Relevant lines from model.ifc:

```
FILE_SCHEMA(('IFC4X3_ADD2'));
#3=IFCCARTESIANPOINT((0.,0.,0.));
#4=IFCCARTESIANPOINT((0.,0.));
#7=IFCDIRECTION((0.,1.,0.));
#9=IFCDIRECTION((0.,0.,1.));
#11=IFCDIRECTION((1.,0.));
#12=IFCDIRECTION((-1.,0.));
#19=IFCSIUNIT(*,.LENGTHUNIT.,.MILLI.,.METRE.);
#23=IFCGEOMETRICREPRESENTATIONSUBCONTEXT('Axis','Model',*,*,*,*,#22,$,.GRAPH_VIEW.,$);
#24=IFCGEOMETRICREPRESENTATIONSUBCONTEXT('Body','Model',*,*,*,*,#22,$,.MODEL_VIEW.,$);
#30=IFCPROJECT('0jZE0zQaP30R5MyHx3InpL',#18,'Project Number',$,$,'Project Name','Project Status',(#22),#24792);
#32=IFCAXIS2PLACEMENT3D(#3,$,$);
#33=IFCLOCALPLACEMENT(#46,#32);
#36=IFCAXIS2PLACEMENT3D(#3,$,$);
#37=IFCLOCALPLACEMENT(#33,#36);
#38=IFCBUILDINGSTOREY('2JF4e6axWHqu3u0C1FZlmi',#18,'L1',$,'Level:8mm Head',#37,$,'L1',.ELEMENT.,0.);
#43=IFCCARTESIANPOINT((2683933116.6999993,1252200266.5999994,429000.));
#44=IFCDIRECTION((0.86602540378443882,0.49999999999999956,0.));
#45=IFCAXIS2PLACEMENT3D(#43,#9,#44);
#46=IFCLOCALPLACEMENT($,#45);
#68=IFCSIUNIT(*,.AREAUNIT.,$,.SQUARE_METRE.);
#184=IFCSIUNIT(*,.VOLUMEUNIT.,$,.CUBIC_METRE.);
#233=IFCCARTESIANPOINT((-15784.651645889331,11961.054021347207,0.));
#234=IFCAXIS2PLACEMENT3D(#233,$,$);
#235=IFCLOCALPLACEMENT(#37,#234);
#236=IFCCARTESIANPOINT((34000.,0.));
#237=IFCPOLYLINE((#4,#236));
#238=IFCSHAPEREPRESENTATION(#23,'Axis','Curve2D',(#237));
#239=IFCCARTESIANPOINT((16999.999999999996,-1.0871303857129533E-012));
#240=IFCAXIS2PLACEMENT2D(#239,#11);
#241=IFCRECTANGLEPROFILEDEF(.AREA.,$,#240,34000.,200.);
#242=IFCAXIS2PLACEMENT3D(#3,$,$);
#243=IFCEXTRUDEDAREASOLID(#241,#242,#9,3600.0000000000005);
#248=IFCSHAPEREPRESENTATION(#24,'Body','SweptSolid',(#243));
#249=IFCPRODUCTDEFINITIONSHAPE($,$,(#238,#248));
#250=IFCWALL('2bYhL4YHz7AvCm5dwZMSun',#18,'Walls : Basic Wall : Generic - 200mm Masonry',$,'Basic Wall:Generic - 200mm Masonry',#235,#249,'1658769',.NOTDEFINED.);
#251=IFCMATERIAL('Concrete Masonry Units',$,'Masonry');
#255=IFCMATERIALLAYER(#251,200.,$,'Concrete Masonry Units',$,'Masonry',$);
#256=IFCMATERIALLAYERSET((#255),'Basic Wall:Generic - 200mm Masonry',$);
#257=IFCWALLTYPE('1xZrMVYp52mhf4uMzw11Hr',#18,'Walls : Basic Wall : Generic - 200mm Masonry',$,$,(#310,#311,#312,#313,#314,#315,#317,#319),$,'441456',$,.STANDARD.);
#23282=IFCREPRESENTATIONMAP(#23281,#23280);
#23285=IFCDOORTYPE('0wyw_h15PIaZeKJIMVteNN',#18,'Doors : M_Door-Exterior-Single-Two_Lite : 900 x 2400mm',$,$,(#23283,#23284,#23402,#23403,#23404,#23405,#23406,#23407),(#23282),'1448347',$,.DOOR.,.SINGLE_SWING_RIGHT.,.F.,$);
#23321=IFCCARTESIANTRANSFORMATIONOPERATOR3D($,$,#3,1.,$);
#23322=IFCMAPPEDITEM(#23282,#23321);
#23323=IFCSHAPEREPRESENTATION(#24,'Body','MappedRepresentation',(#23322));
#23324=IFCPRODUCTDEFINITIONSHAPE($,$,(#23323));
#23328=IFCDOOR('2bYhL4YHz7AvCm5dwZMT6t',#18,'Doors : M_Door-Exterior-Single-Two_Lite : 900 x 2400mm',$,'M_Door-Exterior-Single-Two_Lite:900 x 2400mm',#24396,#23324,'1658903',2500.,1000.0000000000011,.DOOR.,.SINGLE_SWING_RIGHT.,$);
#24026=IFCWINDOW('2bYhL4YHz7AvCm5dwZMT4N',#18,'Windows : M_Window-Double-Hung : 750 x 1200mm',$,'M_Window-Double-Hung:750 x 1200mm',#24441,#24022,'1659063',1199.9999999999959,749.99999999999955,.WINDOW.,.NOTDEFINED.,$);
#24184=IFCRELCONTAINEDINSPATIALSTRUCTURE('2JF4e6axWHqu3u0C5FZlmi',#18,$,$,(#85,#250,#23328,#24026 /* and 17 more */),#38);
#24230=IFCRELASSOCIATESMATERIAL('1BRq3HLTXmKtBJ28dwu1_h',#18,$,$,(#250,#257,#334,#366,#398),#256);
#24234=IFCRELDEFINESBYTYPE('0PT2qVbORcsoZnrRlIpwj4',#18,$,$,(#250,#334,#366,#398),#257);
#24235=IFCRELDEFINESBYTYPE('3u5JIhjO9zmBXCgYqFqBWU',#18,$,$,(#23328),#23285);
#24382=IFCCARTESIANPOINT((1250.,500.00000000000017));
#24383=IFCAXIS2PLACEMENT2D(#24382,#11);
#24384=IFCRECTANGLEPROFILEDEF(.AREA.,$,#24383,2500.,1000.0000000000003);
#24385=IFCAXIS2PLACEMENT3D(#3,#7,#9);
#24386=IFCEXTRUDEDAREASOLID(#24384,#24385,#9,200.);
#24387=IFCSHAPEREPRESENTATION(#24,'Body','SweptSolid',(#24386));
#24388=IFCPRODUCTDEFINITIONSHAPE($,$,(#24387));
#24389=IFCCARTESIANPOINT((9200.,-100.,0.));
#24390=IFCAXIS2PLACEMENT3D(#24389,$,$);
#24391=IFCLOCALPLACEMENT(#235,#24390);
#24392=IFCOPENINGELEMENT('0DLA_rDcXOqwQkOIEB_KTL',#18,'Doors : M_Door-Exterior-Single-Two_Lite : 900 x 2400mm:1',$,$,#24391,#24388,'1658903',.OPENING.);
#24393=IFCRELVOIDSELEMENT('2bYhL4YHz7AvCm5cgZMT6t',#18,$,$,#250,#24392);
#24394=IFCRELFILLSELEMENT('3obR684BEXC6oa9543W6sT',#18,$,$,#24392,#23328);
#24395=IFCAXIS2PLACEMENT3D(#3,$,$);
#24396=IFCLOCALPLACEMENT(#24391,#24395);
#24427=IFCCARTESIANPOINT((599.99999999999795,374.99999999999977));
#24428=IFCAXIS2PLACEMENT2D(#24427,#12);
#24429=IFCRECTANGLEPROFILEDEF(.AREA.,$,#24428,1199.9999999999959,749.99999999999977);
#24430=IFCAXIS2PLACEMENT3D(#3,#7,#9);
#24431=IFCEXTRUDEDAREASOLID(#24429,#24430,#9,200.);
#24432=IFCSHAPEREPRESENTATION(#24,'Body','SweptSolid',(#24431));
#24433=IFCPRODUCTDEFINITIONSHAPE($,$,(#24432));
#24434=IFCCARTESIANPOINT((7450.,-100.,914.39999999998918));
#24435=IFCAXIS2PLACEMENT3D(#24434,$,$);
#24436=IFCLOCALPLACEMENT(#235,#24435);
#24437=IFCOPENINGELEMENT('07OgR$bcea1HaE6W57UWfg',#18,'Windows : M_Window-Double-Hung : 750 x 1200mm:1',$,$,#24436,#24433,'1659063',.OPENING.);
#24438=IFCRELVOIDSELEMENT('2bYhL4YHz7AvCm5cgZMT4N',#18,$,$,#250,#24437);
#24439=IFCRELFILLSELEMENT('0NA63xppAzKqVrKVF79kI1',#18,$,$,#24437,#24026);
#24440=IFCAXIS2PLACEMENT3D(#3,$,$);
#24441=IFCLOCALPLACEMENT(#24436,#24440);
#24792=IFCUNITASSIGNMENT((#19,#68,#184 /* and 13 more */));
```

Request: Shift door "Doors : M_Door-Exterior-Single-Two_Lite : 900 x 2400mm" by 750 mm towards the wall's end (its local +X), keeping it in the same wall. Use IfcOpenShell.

```python
import ifcopenshell
import ifcopenshell.api.geometry
import ifcopenshell.util.placement
import ifcopenshell.util.unit

model = ifcopenshell.open("model.ifc")
unit_scale = ifcopenshell.util.unit.calculate_unit_scale(model)

door = model.by_id(23328)
opening = door.FillsVoids[0].RelatingOpeningElement
wall = opening.VoidsElements[0].RelatingBuildingElement

wall_matrix = ifcopenshell.util.placement.get_local_placement(wall.ObjectPlacement)
shift = wall_matrix[:3, 0] * 0.75 / unit_scale
before = ifcopenshell.util.placement.get_local_placement(door.ObjectPlacement)[:3, 3].copy()

# The door is placed relative to its opening, so it follows when the opening moves.
matrix = ifcopenshell.util.placement.get_local_placement(opening.ObjectPlacement)
matrix[:3, 3] += shift
ifcopenshell.api.geometry.edit_object_placement(
    model, product=opening, matrix=matrix, is_si=False, should_transform_children=True
)

after = ifcopenshell.util.placement.get_local_placement(door.ObjectPlacement)[:3, 3]
print("door moved by", (after - before).round(3) + 0.0)

model.write("model_edited.ifc")
```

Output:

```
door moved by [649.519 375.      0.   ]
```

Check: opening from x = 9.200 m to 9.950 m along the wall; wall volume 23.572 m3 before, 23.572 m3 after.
